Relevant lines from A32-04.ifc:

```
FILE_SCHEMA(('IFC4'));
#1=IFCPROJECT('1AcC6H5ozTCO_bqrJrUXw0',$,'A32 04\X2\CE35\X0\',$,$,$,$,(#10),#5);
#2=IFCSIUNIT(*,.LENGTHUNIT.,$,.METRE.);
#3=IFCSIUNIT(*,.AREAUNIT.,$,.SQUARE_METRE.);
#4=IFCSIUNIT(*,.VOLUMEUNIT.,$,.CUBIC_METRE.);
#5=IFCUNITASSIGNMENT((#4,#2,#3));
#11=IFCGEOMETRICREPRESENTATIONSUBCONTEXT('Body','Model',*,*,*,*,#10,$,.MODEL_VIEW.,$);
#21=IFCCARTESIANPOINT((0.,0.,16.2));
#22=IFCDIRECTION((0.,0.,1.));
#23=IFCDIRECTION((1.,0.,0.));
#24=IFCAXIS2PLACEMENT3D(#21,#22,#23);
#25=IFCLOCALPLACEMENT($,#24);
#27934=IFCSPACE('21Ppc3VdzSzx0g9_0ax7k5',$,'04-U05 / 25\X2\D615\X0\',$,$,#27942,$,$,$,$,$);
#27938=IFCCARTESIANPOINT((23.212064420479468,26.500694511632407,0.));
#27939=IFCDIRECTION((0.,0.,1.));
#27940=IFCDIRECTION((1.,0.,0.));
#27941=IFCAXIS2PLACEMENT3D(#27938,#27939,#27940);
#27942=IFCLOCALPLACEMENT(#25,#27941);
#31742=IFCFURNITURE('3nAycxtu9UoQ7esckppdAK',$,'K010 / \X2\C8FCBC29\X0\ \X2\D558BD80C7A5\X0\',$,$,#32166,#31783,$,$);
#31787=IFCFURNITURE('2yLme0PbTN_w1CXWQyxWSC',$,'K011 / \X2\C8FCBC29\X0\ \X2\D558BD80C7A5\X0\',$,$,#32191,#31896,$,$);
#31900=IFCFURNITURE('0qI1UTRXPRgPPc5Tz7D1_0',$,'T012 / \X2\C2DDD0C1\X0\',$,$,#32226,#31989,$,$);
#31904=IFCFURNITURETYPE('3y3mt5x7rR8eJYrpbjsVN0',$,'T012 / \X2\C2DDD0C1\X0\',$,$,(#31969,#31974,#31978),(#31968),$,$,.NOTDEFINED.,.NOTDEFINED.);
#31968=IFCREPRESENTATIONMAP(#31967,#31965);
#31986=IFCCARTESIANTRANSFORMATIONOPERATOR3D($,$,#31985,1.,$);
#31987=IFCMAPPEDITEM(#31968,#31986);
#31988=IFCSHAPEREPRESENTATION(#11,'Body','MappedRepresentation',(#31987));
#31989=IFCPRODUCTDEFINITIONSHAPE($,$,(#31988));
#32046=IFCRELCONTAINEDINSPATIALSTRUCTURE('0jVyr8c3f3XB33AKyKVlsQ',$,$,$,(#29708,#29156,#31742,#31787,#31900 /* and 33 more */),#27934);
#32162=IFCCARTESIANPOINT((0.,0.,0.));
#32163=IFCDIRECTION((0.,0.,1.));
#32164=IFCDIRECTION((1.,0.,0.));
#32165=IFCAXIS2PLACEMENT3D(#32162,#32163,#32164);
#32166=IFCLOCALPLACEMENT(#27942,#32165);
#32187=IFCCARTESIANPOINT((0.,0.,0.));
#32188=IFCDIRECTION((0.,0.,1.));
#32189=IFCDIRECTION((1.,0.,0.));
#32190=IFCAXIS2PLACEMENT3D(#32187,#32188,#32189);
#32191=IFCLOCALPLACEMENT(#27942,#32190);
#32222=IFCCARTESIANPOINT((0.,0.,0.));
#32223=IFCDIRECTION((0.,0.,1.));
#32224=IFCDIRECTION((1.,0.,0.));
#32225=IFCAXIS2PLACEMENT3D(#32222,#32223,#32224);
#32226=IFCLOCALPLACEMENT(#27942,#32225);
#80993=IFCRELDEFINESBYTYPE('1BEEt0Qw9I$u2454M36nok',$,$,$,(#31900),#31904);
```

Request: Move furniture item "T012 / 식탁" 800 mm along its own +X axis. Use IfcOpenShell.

```python
import ifcopenshell
import ifcopenshell.api.geometry
import ifcopenshell.util.placement

model = ifcopenshell.open("A32-04.ifc")

item = model.by_guid("0qI1UTRXPRgPPc5Tz7D1_0")
matrix = ifcopenshell.util.placement.get_local_placement(item.ObjectPlacement)
matrix[:3, 3] += matrix[:3, 0] * 0.8
ifcopenshell.api.geometry.edit_object_placement(model, product=item, matrix=matrix, is_si=False)

print(ifcopenshell.util.placement.get_local_placement(item.ObjectPlacement).round(3) + 0.0)

model.write("A32-04_rev.ifc")
```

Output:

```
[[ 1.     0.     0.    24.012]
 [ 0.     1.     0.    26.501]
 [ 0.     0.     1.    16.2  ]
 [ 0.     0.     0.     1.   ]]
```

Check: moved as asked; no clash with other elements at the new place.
